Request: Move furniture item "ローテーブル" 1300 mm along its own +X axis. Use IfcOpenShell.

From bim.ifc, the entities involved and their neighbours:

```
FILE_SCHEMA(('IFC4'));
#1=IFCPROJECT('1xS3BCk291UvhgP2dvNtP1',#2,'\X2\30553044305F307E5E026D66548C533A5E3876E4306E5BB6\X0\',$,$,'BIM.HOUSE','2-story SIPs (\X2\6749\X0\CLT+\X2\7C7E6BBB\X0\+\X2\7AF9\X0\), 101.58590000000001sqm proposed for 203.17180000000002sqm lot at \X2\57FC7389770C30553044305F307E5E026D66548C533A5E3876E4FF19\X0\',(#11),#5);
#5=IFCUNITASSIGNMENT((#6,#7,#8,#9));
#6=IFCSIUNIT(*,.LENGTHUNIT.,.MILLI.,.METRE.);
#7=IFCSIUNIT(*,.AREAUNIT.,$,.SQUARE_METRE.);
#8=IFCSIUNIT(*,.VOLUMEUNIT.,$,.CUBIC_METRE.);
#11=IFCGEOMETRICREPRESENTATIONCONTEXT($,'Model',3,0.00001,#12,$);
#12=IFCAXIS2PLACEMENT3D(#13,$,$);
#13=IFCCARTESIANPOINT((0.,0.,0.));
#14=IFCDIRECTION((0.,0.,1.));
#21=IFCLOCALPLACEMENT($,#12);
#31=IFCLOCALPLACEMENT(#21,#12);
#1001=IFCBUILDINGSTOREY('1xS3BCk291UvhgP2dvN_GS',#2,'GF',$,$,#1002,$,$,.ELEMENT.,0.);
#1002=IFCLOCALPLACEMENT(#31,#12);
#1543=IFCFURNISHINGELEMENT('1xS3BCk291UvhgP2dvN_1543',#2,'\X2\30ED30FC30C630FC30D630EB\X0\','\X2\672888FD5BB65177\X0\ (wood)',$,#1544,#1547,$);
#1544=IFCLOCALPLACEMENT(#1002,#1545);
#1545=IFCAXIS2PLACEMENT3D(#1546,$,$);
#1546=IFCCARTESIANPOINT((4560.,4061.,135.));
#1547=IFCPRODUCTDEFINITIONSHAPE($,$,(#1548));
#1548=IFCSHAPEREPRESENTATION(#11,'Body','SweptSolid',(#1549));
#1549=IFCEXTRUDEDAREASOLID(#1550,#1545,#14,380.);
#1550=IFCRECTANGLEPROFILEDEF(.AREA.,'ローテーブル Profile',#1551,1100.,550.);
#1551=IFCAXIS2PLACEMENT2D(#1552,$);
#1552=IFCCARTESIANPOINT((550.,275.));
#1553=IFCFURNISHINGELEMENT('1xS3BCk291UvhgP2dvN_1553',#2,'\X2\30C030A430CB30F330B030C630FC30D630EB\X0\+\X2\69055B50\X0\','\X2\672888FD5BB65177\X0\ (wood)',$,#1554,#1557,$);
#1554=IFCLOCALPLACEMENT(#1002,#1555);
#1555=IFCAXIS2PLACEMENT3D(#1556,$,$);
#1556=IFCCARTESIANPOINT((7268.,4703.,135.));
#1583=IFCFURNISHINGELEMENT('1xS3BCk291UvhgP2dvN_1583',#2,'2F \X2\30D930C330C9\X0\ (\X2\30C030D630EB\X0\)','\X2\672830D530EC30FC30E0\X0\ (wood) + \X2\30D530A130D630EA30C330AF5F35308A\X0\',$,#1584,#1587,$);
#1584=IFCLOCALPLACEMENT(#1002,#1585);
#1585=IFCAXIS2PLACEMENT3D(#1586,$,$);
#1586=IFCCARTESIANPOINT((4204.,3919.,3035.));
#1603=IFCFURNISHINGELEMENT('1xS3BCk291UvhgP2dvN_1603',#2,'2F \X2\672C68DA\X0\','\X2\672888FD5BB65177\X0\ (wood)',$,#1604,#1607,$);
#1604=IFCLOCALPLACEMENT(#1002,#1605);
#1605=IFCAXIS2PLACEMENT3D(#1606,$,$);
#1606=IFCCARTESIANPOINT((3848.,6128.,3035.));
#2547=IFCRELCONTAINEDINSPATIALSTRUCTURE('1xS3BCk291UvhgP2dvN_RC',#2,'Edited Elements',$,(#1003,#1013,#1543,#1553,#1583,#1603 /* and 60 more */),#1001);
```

```python
import ifcopenshell
import ifcopenshell.api.geometry
import ifcopenshell.util.placement

model = ifcopenshell.open("bim.ifc")

item = model.by_guid("1xS3BCk291UvhgP2dvN_1543")
matrix = ifcopenshell.util.placement.get_local_placement(item.ObjectPlacement)
matrix[:3, 3] += matrix[:3, 0] * 1300.0
ifcopenshell.api.geometry.edit_object_placement(model, product=item, matrix=matrix, is_si=False)

print(ifcopenshell.util.placement.get_local_placement(item.ObjectPlacement).round(3) + 0.0)

model.write("bim_edited.ifc")
```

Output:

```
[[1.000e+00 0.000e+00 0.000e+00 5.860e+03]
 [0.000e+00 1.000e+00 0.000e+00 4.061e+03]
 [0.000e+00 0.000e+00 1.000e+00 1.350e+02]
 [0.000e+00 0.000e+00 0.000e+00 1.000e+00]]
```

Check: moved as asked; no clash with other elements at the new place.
